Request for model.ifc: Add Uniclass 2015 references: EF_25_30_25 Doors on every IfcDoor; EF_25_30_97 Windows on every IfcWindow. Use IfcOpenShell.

First a look at what the model holds.

```python
import ifcopenshell

model = ifcopenshell.open("model.ifc")
print(model.schema)
print("classifications:", [c.Name for c in model.by_type("IfcClassification")])
for ifc_class in ("IfcDoor", "IfcRoof", "IfcStair", "IfcWall", "IfcWindow"):
    print(ifc_class, len(model.by_type(ifc_class)))
```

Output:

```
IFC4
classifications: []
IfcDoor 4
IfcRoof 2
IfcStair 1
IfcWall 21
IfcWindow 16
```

```python
import ifcopenshell
import ifcopenshell.api.classification

model = ifcopenshell.open("model.ifc")

system = ifcopenshell.api.classification.add_classification(model, classification="Uniclass 2015")

codes = {
    "IfcDoor": ("EF_25_30_25", "Doors"),
    "IfcWindow": ("EF_25_30_97", "Windows"),
}
for ifc_class, (code, name) in codes.items():
    products = model.by_type(ifc_class)
    ifcopenshell.api.classification.add_reference(
        model, products=products, classification=system, identification=code, name=name
    )
    print(code, len(products))

model.write("model_edited.ifc")
```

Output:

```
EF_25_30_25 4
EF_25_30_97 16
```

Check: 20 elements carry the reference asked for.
